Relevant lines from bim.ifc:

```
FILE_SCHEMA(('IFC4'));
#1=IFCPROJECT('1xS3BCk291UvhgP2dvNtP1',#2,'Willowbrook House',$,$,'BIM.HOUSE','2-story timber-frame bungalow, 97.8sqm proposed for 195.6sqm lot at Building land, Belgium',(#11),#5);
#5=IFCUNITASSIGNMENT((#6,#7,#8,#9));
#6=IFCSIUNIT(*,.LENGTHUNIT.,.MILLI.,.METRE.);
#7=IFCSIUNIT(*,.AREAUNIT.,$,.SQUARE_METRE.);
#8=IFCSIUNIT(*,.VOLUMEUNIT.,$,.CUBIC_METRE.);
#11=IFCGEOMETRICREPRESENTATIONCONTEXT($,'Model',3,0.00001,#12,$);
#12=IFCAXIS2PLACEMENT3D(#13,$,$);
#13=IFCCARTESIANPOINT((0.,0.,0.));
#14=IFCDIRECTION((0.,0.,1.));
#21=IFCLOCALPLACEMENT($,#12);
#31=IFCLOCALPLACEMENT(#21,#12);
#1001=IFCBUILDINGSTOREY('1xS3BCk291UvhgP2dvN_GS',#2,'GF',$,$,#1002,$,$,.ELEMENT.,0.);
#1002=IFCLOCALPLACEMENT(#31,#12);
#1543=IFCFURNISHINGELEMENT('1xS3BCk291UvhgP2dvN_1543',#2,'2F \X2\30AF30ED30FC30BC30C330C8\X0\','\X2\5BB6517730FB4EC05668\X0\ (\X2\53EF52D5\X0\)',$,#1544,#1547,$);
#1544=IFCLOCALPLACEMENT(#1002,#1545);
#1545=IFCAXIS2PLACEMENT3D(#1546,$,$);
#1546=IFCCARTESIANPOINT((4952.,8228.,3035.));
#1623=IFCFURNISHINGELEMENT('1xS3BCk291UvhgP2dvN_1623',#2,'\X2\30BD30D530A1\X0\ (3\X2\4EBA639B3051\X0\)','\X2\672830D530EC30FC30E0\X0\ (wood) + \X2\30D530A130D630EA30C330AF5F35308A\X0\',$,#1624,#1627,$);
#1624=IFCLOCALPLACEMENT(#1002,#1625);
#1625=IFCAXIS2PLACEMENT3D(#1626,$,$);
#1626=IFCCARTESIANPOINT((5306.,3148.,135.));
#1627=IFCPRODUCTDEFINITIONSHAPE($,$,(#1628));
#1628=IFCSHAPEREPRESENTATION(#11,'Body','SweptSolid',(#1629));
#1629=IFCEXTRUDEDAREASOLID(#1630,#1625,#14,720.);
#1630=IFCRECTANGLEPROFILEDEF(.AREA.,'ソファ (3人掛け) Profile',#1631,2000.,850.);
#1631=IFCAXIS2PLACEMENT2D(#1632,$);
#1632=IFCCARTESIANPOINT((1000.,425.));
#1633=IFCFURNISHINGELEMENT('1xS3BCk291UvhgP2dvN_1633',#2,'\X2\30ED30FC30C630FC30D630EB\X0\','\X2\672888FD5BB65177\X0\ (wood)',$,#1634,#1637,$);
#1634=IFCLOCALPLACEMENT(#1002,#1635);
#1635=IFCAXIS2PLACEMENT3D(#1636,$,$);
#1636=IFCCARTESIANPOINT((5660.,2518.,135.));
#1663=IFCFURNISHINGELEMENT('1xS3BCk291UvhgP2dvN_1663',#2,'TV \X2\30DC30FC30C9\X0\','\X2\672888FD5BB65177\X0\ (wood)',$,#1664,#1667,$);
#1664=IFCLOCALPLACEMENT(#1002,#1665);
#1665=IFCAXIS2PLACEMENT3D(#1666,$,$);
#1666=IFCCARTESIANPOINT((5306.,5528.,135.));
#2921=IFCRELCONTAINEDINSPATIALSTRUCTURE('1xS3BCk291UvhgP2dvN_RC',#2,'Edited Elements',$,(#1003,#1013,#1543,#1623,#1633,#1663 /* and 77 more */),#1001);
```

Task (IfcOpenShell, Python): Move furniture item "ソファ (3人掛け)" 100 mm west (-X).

```python
import ifcopenshell
import ifcopenshell.api.geometry
import ifcopenshell.util.placement
import ifcopenshell.util.unit

model = ifcopenshell.open("bim.ifc")
unit_scale = ifcopenshell.util.unit.calculate_unit_scale(model)

item = model.by_id(1623)
matrix = ifcopenshell.util.placement.get_local_placement(item.ObjectPlacement)
matrix[0, 3] -= 0.1 / unit_scale
ifcopenshell.api.geometry.edit_object_placement(model, product=item, matrix=matrix, is_si=False)

print(ifcopenshell.util.placement.get_local_placement(item.ObjectPlacement).round(3) + 0.0)

model.write("bim-out.ifc")
```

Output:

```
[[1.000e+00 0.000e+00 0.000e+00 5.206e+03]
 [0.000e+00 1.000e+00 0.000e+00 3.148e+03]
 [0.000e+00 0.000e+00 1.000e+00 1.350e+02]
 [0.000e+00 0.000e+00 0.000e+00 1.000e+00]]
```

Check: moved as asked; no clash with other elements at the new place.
